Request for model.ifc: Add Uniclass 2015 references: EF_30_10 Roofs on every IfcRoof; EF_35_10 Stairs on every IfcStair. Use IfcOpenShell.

First a look at what the model holds.

```python
import ifcopenshell

model = ifcopenshell.open("model.ifc")
print(model.schema)
print("classifications:", [c.Name for c in model.by_type("IfcClassification")])
for ifc_class in ("IfcDoor", "IfcRoof", "IfcStair", "IfcWall", "IfcWindow"):
    print(ifc_class, len(model.by_type(ifc_class)))
```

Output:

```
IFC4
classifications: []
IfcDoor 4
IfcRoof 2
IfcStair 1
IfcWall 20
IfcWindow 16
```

```python
import ifcopenshell
import ifcopenshell.api.classification

model = ifcopenshell.open("model.ifc")

system = ifcopenshell.api.classification.add_classification(model, classification="Uniclass 2015")

codes = {
    "IfcRoof": ("EF_30_10", "Roofs"),
    "IfcStair": ("EF_35_10", "Stairs"),
}
for ifc_class, (code, name) in codes.items():
    products = model.by_type(ifc_class)
    ifcopenshell.api.classification.add_reference(
        model, products=products, classification=system, identification=code, name=name
    )
    print(code, len(products))

model.write("model-out.ifc")
```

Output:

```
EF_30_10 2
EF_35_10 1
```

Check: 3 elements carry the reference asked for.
